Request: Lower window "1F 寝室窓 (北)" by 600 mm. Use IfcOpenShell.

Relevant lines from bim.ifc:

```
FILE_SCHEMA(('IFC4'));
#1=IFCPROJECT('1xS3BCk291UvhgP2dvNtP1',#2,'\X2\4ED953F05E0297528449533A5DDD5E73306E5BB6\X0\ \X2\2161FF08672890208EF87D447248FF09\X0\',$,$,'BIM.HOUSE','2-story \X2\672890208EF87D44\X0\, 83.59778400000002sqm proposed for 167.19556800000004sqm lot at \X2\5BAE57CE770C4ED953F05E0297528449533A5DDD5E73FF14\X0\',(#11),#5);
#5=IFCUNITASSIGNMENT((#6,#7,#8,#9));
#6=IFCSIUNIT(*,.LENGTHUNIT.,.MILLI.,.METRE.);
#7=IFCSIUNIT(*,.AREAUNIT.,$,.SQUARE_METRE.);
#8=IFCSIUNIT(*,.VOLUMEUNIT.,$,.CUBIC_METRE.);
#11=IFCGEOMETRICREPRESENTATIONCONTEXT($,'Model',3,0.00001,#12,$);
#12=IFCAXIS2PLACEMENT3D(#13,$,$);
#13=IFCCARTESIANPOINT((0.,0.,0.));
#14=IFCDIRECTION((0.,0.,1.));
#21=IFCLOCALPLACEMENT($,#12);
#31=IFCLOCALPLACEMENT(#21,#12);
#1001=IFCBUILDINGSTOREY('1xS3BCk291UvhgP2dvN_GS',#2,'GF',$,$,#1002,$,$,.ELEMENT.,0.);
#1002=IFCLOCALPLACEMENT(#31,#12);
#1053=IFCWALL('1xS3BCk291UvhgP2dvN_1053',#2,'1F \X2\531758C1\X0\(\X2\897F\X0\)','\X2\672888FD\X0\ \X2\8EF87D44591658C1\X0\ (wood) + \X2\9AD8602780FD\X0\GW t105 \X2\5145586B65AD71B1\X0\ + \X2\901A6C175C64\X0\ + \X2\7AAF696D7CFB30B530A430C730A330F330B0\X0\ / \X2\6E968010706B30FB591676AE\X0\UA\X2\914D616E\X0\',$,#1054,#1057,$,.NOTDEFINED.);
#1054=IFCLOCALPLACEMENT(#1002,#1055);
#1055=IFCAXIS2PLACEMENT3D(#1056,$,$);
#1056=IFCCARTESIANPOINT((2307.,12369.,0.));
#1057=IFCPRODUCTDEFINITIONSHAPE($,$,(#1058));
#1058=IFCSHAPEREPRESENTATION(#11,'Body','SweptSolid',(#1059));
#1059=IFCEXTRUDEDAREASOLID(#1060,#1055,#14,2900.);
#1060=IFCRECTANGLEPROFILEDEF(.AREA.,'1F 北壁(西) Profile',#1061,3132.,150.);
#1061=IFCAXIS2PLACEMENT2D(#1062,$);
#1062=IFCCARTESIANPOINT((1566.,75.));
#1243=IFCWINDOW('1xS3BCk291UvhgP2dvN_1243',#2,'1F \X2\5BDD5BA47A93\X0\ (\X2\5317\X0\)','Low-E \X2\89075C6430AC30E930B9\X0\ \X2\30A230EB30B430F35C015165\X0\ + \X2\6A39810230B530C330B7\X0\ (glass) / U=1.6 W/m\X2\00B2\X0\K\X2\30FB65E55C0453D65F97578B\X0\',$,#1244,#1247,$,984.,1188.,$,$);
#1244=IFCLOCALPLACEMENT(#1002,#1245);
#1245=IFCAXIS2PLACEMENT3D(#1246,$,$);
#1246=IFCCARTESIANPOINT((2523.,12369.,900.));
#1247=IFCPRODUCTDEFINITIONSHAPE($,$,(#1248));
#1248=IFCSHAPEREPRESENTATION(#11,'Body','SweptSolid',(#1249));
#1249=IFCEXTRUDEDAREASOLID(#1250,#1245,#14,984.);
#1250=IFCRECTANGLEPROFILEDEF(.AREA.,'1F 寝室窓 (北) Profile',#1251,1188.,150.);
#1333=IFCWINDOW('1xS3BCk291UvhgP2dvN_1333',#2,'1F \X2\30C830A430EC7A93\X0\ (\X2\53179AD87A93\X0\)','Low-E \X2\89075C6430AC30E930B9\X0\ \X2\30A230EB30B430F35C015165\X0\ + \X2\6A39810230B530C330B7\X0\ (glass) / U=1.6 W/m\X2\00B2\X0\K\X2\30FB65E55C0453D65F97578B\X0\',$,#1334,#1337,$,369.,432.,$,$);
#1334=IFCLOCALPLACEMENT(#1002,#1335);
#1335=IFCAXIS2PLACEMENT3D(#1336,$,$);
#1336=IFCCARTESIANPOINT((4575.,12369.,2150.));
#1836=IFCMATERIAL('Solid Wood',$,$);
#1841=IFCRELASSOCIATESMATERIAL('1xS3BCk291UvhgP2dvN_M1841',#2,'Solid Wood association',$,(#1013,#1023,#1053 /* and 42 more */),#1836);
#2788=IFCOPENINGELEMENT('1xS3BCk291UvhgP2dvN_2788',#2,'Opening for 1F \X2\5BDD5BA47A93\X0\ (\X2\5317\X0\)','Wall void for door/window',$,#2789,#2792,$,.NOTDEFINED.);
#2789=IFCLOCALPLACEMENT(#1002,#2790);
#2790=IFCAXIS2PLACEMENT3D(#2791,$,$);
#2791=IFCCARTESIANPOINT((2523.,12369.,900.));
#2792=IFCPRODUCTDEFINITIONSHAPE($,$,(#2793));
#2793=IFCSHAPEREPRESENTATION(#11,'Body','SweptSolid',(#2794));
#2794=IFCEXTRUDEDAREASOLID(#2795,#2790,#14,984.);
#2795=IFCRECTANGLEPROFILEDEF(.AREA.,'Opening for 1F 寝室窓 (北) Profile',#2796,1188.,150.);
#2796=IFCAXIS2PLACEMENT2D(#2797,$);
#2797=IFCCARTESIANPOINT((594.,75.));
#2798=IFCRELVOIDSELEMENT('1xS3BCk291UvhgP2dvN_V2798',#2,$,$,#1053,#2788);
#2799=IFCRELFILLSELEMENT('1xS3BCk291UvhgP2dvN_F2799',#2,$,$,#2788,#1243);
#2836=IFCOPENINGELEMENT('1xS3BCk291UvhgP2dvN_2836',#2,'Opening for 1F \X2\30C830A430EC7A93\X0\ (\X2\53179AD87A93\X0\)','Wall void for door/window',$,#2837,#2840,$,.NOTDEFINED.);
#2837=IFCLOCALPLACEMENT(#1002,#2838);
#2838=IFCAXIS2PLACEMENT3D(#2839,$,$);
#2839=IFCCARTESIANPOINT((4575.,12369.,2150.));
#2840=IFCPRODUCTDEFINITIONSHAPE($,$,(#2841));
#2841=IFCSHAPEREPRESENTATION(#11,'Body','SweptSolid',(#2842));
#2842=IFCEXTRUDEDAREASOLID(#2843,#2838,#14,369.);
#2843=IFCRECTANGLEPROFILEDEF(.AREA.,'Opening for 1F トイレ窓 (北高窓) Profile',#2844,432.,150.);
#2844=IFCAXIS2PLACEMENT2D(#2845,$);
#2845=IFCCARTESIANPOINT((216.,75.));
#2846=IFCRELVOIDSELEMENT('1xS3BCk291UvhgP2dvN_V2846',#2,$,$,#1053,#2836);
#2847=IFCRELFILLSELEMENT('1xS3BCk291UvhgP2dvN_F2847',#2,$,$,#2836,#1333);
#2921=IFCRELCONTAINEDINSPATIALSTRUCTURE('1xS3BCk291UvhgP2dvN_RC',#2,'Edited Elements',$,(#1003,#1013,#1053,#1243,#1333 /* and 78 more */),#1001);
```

```python
import numpy as np
import ifcopenshell
import ifcopenshell.api.geometry
import ifcopenshell.util.placement
import ifcopenshell.util.unit

model = ifcopenshell.open("bim.ifc")
unit_scale = ifcopenshell.util.unit.calculate_unit_scale(model)

window = model.by_guid("1xS3BCk291UvhgP2dvN_1243")
opening = window.FillsVoids[0].RelatingOpeningElement
dz = -600.0

shift = np.array([0.0, 0.0, dz])
# The window is not placed relative to its opening, so move both.
for product in (opening, window):
    matrix = ifcopenshell.util.placement.get_local_placement(product.ObjectPlacement)
    matrix[:3, 3] += shift
    ifcopenshell.api.geometry.edit_object_placement(model, product=product, matrix=matrix, is_si=False)

print(f"moved by {dz * unit_scale:+.3f} m")

model.write("bim_updated.ifc")
```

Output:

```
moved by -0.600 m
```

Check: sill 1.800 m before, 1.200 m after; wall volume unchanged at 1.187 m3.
